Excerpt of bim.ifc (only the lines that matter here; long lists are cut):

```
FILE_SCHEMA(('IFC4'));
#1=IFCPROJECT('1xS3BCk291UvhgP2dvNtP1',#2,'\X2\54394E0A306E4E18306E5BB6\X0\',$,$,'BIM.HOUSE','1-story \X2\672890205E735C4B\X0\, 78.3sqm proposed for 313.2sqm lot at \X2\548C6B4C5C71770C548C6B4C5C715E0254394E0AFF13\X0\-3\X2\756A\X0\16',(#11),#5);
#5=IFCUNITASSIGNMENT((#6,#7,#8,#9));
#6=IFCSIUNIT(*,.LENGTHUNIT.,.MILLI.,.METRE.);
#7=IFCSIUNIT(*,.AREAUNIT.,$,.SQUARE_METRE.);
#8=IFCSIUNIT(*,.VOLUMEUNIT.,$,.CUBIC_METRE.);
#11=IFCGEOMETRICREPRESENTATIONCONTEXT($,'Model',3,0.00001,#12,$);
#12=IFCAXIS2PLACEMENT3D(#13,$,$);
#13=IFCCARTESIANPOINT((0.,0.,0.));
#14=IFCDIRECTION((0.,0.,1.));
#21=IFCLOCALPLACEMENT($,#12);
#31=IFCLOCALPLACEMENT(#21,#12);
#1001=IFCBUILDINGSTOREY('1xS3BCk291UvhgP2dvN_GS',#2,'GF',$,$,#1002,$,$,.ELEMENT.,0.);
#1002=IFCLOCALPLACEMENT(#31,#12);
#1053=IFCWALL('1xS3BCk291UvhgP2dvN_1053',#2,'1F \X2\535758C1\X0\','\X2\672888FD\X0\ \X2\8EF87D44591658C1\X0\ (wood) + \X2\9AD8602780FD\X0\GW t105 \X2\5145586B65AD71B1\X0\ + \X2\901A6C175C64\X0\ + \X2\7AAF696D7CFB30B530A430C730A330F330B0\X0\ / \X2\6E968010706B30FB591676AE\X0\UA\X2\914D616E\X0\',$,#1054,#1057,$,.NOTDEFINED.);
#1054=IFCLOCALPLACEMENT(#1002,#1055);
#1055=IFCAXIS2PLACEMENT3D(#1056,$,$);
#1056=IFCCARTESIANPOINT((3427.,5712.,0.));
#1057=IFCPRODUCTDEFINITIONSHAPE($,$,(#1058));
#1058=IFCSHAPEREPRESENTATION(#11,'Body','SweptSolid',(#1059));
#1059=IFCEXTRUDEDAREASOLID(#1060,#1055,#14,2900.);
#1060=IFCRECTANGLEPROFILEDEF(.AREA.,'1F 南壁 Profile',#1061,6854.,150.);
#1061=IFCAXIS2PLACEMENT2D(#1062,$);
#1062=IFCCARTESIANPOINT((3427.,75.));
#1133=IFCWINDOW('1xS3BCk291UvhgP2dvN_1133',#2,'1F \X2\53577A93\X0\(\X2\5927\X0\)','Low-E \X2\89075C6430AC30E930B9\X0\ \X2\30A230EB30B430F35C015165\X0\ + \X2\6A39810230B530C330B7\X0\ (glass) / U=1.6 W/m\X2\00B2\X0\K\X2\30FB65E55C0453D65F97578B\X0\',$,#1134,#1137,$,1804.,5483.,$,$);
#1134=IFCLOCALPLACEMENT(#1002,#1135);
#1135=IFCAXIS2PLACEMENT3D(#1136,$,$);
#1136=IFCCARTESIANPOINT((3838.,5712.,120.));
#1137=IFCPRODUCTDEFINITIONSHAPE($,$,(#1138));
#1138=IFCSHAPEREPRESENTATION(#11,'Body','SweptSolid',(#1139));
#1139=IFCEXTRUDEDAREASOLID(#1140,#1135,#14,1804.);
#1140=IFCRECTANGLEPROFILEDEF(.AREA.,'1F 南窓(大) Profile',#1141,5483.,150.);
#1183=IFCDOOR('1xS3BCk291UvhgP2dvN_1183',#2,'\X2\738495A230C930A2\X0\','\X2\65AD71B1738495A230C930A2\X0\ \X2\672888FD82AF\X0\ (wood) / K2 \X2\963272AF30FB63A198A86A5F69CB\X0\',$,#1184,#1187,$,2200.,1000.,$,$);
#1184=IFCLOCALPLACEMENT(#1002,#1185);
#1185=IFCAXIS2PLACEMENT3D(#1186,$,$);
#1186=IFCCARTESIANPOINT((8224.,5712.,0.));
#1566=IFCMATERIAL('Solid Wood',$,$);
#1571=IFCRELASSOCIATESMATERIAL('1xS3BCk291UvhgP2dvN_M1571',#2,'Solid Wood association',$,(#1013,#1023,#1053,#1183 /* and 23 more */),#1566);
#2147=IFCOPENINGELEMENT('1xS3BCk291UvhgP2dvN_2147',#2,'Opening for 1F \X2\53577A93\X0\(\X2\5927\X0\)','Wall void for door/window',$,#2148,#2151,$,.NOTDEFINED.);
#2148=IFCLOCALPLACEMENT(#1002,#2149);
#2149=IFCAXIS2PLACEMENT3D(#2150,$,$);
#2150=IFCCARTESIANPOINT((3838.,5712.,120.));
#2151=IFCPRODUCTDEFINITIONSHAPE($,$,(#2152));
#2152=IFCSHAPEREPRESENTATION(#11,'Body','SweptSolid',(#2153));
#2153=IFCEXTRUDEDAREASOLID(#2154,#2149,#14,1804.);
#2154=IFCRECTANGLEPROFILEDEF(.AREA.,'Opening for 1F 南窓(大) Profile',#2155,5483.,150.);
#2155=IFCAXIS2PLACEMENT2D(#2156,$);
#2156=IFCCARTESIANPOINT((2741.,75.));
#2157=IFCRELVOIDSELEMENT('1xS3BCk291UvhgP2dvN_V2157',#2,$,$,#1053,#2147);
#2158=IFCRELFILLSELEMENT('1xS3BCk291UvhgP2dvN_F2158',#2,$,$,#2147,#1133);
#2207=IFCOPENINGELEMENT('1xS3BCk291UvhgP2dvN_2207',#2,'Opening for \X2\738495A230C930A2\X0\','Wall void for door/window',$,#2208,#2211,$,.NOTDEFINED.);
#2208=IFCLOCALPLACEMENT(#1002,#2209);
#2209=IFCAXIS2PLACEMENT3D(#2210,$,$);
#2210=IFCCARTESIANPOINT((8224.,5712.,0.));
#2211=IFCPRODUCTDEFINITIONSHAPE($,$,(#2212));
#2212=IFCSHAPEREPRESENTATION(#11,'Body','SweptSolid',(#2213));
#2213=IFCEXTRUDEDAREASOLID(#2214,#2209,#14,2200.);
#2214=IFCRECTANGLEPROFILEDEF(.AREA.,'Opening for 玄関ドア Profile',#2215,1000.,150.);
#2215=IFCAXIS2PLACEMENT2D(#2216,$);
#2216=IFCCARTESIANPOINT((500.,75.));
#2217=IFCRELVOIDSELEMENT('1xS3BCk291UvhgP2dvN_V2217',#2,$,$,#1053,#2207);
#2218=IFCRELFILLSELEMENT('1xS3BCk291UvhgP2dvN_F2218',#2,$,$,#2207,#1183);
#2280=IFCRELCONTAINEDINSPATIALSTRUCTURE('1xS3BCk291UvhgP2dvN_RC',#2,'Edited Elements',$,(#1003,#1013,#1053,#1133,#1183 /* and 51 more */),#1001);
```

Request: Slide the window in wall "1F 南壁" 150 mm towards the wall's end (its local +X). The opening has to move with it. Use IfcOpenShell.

```python
import ifcopenshell
import ifcopenshell.api.geometry
import ifcopenshell.util.placement

model = ifcopenshell.open("bim.ifc")

window = model.by_guid("1xS3BCk291UvhgP2dvN_1133")
opening = window.FillsVoids[0].RelatingOpeningElement
wall = opening.VoidsElements[0].RelatingBuildingElement

wall_matrix = ifcopenshell.util.placement.get_local_placement(wall.ObjectPlacement)
shift = wall_matrix[:3, 0] * 150.0
before = ifcopenshell.util.placement.get_local_placement(window.ObjectPlacement)[:3, 3].copy()

# The window is not placed relative to its opening, so move both.
for product in (opening, window):
    matrix = ifcopenshell.util.placement.get_local_placement(product.ObjectPlacement)
    matrix[:3, 3] += shift
    ifcopenshell.api.geometry.edit_object_placement(model, product=product, matrix=matrix, is_si=False)

after = ifcopenshell.util.placement.get_local_placement(window.ObjectPlacement)[:3, 3]
print("window moved by", (after - before).round(3) + 0.0)

model.write("bim_updated.ifc")
```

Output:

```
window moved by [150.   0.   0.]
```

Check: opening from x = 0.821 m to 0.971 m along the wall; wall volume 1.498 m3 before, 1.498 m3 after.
